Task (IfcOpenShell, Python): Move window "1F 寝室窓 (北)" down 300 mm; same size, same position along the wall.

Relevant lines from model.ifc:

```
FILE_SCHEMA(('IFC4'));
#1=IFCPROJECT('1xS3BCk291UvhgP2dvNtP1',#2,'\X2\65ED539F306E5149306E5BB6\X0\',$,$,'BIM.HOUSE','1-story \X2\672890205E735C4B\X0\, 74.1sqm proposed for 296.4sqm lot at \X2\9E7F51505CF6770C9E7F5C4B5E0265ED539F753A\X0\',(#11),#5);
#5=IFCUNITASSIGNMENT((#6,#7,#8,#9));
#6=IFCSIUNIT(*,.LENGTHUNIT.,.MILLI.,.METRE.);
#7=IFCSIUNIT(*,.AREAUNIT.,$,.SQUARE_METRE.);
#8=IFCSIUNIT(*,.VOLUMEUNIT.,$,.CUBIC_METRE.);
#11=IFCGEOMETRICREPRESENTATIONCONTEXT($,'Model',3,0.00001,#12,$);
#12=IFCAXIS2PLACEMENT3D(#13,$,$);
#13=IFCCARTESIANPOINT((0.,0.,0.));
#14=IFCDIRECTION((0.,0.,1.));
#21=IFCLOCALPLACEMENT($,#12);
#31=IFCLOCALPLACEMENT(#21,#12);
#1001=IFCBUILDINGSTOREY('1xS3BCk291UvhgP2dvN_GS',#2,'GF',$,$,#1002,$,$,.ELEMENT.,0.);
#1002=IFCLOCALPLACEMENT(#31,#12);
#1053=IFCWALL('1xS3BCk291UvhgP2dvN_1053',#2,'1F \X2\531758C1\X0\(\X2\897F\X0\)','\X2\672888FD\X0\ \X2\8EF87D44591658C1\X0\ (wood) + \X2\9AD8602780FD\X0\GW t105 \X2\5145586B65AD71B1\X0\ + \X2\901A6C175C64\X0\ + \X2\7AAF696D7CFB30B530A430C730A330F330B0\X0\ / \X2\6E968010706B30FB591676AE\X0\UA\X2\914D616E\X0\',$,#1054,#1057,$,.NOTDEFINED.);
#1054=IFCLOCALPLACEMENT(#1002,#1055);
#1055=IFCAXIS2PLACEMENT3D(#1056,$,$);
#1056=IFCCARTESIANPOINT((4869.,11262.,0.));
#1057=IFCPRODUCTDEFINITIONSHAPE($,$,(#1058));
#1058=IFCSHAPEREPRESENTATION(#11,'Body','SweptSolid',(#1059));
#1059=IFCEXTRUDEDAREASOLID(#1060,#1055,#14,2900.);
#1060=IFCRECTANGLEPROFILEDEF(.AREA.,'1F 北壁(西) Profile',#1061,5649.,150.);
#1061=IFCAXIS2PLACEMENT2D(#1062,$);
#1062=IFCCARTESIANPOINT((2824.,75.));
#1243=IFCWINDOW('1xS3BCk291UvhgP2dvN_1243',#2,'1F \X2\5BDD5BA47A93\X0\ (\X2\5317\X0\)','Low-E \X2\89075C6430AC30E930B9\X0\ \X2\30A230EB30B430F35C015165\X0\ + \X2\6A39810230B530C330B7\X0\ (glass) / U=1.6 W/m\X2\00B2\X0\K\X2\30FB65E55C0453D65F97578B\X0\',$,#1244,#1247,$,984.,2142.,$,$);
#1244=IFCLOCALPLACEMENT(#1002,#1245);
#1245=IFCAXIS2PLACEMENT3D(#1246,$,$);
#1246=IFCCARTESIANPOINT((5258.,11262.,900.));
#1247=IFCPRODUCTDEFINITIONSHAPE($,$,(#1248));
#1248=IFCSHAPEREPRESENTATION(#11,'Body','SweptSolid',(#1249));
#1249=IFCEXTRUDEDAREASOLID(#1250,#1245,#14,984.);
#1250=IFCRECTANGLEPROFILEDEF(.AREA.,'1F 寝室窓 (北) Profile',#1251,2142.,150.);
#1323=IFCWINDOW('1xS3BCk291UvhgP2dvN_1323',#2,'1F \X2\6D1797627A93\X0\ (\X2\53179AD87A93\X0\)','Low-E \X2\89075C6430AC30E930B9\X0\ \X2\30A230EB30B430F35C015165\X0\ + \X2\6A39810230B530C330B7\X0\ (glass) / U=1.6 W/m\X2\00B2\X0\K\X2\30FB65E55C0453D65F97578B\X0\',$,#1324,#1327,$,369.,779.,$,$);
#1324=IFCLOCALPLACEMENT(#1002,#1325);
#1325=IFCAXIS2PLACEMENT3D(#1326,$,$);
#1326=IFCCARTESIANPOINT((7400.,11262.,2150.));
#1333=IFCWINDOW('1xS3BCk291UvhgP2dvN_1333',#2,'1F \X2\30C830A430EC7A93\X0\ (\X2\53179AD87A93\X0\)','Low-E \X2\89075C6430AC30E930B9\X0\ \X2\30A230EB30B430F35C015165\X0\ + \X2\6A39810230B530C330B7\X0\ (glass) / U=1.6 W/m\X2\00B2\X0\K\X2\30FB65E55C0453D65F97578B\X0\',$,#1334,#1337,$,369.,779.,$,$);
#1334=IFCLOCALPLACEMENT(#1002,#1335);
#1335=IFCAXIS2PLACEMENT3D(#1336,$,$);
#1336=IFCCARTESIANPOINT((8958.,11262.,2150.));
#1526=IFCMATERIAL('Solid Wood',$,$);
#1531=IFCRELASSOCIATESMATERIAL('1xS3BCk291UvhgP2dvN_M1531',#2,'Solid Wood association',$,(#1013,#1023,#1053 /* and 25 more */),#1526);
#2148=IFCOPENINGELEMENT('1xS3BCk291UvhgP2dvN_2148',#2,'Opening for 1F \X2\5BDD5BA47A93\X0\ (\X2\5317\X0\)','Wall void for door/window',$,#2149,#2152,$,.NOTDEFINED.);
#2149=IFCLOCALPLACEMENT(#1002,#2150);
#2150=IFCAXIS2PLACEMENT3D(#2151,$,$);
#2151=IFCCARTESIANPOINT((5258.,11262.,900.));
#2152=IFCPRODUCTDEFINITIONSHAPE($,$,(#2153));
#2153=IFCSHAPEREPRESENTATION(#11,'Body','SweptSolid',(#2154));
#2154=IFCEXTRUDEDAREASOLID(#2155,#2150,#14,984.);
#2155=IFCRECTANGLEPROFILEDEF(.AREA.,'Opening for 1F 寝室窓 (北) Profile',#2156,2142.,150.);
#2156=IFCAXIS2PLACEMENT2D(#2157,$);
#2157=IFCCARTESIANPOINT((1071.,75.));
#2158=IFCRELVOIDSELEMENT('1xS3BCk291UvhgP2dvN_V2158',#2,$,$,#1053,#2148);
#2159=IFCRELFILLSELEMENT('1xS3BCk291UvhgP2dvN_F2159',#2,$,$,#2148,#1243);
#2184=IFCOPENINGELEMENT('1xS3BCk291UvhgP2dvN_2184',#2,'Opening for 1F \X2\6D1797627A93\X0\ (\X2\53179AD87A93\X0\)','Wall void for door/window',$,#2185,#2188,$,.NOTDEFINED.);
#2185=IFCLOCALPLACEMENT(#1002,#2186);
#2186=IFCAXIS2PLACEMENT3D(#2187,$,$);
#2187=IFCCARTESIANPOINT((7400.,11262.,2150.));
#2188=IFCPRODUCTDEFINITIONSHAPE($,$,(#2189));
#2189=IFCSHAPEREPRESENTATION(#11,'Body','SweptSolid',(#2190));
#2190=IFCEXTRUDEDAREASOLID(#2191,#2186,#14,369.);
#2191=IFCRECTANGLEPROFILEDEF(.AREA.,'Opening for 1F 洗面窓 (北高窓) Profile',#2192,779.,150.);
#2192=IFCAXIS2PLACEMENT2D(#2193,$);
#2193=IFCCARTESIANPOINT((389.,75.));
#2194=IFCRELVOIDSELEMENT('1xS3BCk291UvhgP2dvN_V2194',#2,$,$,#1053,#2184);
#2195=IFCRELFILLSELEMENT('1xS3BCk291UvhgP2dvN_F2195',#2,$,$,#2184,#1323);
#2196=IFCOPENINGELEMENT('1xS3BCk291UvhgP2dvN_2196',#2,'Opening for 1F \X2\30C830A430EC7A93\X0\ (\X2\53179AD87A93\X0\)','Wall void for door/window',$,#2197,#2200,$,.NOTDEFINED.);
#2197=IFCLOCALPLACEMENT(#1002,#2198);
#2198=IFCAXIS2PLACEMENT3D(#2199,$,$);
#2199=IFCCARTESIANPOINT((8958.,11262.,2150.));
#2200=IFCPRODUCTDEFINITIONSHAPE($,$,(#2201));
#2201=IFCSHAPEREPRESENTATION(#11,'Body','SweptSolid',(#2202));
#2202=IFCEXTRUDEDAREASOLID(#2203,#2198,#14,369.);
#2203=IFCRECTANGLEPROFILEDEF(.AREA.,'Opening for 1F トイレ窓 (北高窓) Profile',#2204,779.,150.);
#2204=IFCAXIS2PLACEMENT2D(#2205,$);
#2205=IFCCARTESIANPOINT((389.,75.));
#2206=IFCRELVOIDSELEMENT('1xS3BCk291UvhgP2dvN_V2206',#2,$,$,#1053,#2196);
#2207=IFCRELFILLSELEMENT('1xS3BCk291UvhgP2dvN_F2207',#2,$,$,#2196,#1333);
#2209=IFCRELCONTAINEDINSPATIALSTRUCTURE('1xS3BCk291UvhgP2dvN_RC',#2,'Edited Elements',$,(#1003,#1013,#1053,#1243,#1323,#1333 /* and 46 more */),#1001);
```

```python
import numpy as np
import ifcopenshell
import ifcopenshell.api.geometry
import ifcopenshell.util.placement
import ifcopenshell.util.unit

model = ifcopenshell.open("model.ifc")
unit_scale = ifcopenshell.util.unit.calculate_unit_scale(model)

window = model.by_guid("1xS3BCk291UvhgP2dvN_1243")
opening = window.FillsVoids[0].RelatingOpeningElement
dz = -0.3 / unit_scale

shift = np.array([0.0, 0.0, dz])
# The window is not placed relative to its opening, so move both.
for product in (opening, window):
    matrix = ifcopenshell.util.placement.get_local_placement(product.ObjectPlacement)
    matrix[:3, 3] += shift
    ifcopenshell.api.geometry.edit_object_placement(model, product=product, matrix=matrix, is_si=False)

print(f"moved by {dz * unit_scale:+.3f} m")

model.write("model_edited.ifc")
```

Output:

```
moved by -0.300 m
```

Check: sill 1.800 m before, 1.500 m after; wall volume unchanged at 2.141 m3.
